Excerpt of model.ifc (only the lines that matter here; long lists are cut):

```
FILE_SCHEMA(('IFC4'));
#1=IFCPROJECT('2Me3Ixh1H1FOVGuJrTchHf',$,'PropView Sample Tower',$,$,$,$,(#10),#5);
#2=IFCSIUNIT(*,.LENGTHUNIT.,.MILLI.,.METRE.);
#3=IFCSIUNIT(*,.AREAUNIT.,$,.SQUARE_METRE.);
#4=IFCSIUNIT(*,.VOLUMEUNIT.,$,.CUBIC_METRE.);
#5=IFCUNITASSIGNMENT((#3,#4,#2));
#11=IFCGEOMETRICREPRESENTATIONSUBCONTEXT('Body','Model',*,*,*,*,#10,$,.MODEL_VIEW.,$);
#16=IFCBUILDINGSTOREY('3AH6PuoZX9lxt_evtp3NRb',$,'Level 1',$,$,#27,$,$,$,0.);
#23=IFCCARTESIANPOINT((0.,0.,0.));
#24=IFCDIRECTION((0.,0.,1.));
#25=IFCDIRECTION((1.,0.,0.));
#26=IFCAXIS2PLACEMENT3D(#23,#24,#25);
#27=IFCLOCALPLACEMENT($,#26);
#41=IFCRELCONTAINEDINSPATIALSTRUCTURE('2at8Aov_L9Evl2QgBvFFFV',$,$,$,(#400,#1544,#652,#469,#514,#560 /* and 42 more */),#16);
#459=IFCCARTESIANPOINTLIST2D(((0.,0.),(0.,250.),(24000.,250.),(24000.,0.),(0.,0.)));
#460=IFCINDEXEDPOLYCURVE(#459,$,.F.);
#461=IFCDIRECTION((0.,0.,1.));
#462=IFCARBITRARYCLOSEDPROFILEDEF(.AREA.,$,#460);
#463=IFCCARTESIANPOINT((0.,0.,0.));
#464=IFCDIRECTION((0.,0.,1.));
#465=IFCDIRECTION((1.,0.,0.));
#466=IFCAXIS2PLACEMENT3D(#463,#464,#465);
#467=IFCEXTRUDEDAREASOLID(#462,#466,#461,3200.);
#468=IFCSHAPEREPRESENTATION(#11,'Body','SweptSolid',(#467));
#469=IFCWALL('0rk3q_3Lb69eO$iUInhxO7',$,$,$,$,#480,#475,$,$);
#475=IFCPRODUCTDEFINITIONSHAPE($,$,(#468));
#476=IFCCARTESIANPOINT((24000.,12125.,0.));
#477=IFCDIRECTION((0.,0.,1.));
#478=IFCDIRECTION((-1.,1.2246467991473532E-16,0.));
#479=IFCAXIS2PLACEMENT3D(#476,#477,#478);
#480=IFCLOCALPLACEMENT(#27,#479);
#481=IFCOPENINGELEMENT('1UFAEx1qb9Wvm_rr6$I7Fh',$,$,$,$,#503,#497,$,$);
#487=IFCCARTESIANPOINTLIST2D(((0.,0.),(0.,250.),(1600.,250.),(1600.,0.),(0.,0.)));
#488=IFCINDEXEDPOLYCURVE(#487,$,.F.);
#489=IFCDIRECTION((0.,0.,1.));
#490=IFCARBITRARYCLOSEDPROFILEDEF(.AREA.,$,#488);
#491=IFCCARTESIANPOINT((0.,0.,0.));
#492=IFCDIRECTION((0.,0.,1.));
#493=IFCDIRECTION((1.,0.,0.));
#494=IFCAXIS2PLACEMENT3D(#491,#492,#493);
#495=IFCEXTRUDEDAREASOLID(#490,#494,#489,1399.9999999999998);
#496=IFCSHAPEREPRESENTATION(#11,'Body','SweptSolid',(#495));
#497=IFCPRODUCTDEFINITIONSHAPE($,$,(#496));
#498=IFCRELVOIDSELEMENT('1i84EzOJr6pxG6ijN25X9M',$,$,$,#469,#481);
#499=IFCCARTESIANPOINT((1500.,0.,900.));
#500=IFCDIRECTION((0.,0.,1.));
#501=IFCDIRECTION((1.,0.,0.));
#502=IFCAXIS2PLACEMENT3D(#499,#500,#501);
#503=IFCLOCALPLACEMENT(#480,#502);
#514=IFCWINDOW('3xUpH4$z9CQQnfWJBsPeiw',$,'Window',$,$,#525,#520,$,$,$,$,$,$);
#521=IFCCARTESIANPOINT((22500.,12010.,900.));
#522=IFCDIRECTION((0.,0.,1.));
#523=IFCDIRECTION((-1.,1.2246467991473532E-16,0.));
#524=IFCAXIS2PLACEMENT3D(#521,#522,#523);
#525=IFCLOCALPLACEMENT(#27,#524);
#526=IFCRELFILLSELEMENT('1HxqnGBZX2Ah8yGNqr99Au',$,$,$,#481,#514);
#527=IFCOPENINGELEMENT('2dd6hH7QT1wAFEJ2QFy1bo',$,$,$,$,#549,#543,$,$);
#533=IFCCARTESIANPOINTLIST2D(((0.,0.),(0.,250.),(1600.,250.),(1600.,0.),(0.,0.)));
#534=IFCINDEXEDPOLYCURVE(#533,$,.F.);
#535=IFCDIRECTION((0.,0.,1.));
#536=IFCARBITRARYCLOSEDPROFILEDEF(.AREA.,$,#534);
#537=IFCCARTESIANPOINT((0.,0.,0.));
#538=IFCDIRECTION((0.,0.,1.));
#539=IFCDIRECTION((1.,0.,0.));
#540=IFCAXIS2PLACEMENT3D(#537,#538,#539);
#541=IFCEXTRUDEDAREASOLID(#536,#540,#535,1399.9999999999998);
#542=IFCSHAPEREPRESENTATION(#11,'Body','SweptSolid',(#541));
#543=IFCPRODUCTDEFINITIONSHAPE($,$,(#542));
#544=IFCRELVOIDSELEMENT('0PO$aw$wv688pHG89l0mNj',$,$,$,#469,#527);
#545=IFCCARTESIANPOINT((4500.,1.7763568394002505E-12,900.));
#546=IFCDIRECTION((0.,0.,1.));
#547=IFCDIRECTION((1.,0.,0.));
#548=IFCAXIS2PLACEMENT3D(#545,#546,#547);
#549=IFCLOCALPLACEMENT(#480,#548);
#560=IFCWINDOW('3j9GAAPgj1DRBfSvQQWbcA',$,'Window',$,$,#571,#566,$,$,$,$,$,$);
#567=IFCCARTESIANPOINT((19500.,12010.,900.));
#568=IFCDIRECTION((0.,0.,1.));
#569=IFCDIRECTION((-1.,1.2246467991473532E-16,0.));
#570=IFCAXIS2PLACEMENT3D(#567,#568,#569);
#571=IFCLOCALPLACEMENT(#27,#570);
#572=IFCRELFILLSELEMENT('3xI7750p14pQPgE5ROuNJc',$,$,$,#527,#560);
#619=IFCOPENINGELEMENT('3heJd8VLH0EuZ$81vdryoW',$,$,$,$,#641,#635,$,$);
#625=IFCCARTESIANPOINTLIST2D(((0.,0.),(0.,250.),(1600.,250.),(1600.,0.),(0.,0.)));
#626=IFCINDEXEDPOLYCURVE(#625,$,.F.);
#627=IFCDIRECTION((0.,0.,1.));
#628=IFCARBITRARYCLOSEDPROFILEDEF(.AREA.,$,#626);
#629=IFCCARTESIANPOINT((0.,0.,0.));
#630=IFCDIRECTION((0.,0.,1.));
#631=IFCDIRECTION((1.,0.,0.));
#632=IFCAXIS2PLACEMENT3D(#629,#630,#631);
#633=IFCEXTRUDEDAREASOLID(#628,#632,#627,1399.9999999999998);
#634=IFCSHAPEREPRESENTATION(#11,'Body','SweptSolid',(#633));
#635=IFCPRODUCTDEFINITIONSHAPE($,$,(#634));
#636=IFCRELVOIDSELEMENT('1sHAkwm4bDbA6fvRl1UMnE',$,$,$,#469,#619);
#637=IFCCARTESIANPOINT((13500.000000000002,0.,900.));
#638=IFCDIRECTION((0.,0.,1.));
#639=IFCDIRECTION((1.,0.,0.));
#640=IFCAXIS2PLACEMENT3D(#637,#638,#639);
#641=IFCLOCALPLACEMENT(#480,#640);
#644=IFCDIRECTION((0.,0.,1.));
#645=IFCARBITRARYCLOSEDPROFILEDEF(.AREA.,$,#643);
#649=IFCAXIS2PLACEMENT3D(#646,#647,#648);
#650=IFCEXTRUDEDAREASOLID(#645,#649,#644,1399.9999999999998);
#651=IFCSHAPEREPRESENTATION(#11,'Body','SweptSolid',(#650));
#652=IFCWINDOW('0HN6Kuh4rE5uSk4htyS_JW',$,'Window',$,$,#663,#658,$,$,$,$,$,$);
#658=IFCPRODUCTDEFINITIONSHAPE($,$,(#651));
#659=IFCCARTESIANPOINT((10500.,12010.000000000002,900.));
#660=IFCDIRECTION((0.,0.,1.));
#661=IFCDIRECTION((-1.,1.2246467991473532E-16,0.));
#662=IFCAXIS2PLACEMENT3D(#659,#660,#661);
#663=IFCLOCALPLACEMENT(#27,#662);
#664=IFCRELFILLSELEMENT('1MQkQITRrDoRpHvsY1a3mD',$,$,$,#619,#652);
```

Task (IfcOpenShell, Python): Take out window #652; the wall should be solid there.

```python
import ifcopenshell
import ifcopenshell.api.feature
import ifcopenshell.api.root
import ifcopenshell.geom
import ifcopenshell.util.shape

model = ifcopenshell.open("model.ifc")
settings = ifcopenshell.geom.settings()


def volume(element):
    """Net volume in cubic metres, openings subtracted."""
    shape = ifcopenshell.geom.create_shape(settings, element)
    return ifcopenshell.util.shape.get_volume(shape.geometry)


window = model.by_guid("0HN6Kuh4rE5uSk4htyS_JW")
opening = window.FillsVoids[0].RelatingOpeningElement
wall = opening.VoidsElements[0].RelatingBuildingElement
before = volume(wall)

ifcopenshell.api.root.remove_product(model, product=window)
ifcopenshell.api.feature.remove_feature(model, feature=opening)

after = volume(wall)

print(f"wall volume {before:.3f} -> {after:.3f} m3")

model.write("model_v2.ifc")
```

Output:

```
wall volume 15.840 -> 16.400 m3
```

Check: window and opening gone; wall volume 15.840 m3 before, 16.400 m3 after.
